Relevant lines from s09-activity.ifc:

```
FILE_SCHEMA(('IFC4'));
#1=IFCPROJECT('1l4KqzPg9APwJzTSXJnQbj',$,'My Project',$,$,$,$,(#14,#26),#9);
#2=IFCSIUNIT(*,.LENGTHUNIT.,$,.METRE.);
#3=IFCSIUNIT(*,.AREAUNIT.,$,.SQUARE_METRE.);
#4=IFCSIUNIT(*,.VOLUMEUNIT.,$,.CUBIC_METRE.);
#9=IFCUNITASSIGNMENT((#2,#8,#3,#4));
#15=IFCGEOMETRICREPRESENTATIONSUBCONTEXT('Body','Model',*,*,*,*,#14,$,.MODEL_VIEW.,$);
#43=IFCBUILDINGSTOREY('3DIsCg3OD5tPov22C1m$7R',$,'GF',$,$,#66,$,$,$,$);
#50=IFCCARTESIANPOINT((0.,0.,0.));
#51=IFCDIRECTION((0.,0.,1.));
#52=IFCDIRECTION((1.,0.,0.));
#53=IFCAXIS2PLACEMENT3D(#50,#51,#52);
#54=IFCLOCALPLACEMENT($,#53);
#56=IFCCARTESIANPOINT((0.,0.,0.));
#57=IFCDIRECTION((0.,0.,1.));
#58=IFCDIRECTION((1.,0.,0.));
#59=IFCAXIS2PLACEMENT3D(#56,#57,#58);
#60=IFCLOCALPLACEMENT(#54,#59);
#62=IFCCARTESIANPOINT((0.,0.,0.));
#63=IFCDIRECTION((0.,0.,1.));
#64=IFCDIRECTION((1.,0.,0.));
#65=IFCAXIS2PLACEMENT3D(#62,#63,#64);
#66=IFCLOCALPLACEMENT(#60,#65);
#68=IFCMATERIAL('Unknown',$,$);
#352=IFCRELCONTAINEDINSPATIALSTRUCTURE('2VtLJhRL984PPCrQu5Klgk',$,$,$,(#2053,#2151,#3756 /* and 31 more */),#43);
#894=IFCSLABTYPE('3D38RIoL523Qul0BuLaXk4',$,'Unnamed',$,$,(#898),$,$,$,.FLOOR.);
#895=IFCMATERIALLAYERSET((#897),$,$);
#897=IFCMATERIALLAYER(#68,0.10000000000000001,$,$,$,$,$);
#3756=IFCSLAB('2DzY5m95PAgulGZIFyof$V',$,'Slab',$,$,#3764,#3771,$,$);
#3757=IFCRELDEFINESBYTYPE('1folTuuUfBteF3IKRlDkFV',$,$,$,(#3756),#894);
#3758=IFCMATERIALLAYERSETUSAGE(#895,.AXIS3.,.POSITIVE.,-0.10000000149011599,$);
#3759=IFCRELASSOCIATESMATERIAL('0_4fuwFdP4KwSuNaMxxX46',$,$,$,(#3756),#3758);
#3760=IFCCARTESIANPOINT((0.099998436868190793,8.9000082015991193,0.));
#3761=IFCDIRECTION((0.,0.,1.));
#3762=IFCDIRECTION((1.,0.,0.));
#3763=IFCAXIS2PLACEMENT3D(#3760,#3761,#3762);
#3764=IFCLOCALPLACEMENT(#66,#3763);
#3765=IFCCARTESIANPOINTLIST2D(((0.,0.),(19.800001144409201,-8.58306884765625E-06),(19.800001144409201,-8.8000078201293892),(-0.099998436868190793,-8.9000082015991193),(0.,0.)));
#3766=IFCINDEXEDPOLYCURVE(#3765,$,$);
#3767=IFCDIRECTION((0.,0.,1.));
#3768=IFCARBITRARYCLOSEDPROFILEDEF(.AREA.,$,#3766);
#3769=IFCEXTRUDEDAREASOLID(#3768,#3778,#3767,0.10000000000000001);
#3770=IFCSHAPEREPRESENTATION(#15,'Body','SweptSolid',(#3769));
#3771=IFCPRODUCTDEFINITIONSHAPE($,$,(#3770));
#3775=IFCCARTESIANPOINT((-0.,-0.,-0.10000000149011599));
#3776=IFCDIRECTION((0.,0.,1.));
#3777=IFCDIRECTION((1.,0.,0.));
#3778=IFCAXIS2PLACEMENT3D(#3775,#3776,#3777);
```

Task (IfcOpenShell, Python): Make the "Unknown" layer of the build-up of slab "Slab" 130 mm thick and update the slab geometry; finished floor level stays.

```python
import ifcopenshell
import ifcopenshell.util.element
import ifcopenshell.util.representation
import ifcopenshell.util.unit

model = ifcopenshell.open("s09-activity.ifc")
unit_scale = ifcopenshell.util.unit.calculate_unit_scale(model)

layer_set = model.by_id(895)
layer = next(l for l in layer_set.MaterialLayers if l.Material and l.Material.Name == "Unknown")
change = 0.13 / unit_scale - layer.LayerThickness
layer.LayerThickness += change

# Geometry does not follow the layer set by itself.
slabs = [e for e in ifcopenshell.util.element.get_elements_by_material(model, layer_set) if e.is_a("IfcSlab")]
for slab in sorted(slabs, key=lambda e: e.id()):
    body = ifcopenshell.util.representation.get_representation(slab, "Model", "Body")
    solid = body.Items[0]
    old_depth = solid.Depth
    solid.Depth += change
    # Extruded upwards: lower the start of the extrusion so the top stays.
    x, y, z = solid.Position.Location.Coordinates
    solid.Position.Location = model.createIfcCartesianPoint((x, y, z - change))
    print(slab.id(), f"{old_depth:g} -> {solid.Depth:g}")

# The layers are counted up from the underside, which has moved.
for usage in {ifcopenshell.util.element.get_material(slab) for slab in slabs}:
    usage.OffsetFromReferenceLine -= change

model.write("s09-activity_v2.ifc")
```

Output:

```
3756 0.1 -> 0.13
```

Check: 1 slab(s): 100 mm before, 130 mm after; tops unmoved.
